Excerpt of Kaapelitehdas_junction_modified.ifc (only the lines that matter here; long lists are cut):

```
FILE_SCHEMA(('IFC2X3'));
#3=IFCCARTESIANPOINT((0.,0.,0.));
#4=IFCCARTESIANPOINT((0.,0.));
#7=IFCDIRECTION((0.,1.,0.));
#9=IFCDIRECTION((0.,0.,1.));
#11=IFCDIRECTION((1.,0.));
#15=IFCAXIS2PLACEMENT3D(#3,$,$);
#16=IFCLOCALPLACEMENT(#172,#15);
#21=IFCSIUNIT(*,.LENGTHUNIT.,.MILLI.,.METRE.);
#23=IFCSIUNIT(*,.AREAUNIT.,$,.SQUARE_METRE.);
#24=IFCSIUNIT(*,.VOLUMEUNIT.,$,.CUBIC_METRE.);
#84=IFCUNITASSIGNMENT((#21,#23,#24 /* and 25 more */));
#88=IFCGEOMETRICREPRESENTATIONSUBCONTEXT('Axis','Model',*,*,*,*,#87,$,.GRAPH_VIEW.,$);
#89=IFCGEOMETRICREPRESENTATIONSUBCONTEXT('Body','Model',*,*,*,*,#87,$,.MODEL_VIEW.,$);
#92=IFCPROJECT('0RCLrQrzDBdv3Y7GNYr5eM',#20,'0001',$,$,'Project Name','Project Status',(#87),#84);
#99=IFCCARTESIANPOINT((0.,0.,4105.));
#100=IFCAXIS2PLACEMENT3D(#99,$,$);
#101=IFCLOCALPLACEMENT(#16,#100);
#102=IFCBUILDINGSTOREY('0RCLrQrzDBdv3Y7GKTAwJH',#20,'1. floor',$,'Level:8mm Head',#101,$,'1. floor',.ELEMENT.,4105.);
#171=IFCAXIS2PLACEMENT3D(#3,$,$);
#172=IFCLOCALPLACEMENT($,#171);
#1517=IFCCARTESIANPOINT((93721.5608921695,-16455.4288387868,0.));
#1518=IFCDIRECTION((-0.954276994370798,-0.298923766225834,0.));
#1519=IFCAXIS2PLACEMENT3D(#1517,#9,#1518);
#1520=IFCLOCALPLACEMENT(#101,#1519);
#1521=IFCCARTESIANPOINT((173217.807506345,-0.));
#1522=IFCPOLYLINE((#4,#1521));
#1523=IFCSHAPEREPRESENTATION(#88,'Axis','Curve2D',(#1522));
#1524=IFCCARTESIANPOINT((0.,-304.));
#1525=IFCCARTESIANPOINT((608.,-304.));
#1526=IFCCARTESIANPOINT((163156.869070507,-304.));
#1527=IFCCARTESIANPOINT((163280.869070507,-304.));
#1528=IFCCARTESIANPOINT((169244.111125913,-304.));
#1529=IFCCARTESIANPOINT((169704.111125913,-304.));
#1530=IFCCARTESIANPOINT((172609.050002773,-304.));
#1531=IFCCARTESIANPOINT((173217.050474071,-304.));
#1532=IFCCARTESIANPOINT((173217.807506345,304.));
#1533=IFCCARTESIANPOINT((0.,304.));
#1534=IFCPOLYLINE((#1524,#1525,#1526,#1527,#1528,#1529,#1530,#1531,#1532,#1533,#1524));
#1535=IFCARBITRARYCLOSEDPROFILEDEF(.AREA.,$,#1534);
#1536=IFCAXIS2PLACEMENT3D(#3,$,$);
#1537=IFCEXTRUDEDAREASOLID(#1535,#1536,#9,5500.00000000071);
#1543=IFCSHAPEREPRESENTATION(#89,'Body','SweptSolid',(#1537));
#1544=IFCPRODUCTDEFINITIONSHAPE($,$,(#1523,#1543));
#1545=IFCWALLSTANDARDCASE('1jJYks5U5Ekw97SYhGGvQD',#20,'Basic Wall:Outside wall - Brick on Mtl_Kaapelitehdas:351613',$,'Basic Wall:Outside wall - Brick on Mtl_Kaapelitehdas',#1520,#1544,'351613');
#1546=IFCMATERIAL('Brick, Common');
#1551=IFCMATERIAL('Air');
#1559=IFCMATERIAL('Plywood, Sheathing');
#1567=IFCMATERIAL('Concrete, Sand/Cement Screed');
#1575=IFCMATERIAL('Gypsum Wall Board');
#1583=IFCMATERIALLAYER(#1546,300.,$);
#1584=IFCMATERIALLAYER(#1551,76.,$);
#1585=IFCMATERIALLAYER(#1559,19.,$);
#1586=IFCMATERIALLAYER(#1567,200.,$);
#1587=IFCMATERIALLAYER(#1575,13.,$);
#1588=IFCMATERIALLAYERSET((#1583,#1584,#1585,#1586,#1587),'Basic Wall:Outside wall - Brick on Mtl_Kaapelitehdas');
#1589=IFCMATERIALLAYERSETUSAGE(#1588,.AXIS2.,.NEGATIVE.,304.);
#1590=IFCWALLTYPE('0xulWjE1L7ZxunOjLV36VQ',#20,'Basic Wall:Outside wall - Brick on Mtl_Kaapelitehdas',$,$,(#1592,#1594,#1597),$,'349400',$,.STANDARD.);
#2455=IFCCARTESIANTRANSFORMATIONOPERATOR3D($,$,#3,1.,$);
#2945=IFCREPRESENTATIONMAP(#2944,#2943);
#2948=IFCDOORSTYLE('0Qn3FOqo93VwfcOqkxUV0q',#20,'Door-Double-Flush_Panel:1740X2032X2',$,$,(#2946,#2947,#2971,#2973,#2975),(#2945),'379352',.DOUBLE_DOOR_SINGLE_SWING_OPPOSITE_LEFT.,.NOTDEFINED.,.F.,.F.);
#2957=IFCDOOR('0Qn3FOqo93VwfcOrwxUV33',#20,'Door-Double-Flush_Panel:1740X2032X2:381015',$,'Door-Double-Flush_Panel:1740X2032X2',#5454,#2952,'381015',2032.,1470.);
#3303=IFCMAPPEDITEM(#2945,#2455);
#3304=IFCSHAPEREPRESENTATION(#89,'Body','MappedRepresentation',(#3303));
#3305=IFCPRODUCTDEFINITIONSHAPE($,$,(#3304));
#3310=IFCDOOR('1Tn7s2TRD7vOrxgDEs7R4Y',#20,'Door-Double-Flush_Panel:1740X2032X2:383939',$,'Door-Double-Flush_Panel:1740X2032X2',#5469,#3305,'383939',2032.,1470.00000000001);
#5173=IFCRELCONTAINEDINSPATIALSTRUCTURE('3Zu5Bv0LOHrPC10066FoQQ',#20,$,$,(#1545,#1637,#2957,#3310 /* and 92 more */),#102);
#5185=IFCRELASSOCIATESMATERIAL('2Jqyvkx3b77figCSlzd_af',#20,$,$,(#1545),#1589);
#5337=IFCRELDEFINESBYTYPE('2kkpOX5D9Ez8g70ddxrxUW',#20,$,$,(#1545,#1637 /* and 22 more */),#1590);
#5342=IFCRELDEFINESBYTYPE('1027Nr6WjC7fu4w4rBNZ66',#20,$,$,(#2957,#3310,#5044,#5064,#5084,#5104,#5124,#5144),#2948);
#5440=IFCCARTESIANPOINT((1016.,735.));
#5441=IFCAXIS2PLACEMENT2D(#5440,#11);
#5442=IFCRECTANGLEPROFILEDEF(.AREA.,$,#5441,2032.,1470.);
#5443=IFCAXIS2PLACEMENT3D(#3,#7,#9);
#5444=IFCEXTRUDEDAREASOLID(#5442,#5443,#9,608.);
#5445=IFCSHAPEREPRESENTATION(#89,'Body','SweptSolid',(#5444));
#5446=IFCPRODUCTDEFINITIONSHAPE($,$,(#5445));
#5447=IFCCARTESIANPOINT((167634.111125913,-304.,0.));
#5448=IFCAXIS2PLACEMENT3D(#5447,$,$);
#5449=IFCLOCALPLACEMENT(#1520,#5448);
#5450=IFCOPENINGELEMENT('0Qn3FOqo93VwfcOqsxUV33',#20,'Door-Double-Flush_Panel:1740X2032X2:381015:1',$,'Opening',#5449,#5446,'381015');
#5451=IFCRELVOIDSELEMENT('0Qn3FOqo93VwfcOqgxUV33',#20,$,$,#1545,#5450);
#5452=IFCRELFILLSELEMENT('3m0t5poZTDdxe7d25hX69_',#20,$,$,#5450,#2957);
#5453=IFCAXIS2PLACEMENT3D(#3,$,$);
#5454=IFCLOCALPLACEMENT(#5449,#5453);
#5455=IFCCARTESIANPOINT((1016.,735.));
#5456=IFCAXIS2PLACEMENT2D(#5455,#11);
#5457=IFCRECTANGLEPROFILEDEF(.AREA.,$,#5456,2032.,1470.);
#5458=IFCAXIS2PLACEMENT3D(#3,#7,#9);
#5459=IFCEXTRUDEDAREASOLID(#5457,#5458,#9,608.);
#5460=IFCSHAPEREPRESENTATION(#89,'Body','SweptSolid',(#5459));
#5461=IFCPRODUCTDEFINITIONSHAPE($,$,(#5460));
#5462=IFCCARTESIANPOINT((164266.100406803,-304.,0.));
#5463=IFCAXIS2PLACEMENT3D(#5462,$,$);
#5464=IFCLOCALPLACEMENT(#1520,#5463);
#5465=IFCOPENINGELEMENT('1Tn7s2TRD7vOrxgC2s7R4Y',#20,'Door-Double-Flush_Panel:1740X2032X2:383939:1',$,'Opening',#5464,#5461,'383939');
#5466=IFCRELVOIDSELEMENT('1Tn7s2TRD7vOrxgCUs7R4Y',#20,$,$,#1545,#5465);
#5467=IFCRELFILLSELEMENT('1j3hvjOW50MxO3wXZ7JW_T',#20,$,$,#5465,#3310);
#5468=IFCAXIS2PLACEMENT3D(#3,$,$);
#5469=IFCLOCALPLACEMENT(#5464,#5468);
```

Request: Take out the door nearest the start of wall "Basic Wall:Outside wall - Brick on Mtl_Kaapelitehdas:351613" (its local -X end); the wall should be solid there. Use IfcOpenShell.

```python
import ifcopenshell
import ifcopenshell.api.feature
import ifcopenshell.api.root
import ifcopenshell.geom
import ifcopenshell.util.shape

model = ifcopenshell.open("Kaapelitehdas_junction_modified.ifc")
settings = ifcopenshell.geom.settings()


def volume(element):
    """Net volume in cubic metres, openings subtracted."""
    shape = ifcopenshell.geom.create_shape(settings, element)
    return ifcopenshell.util.shape.get_volume(shape.geometry)


door = model.by_guid("1Tn7s2TRD7vOrxgDEs7R4Y")
opening = door.FillsVoids[0].RelatingOpeningElement
wall = opening.VoidsElements[0].RelatingBuildingElement
before = volume(wall)

ifcopenshell.api.root.remove_product(model, product=door)
ifcopenshell.api.feature.remove_feature(model, feature=opening)

after = volume(wall)

print(f"wall volume {before:.3f} -> {after:.3f} m3")

model.write("Kaapelitehdas_junction_modified_edited.ifc")
```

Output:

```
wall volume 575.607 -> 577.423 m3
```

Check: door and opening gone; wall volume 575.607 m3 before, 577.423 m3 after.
